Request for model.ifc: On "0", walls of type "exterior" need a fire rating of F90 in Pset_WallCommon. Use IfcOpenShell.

First a look at what the model holds.

```python
import ifcopenshell
import ifcopenshell.util.element

model = ifcopenshell.open("model.ifc")
print(model.schema)
storey = next(s for s in model.by_type("IfcBuildingStorey") if s.Name == "0")
walls = [e for e in ifcopenshell.util.element.get_decomposition(storey) if e.is_a("IfcWall")]
seen = {}
for e in walls:
    element_type = ifcopenshell.util.element.get_type(e)
    key = (element_type.Name if element_type != e and element_type else None, ifcopenshell.util.element.get_pset(e, "Pset_WallCommon", "FireRating"))
    seen[key] = seen.get(key, 0) + 1
for (name, value), count in sorted(seen.items(), key=str):
    print(count, "x", name, "|", value)
```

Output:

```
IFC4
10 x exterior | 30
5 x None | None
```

```python
import ifcopenshell
import ifcopenshell.api.pset
import ifcopenshell.util.element

model = ifcopenshell.open("model.ifc")

storey = next(s for s in model.by_type("IfcBuildingStorey") if s.Name == "0")
walls = [e for e in ifcopenshell.util.element.get_decomposition(storey) if e.is_a("IfcWall")]

count = 0
for e in walls:
    element_type = ifcopenshell.util.element.get_type(e)
    if element_type in (None, e) or element_type.Name != "exterior":
        continue
    # add_pset returns the element's existing set when there is one.
    pset = ifcopenshell.api.pset.add_pset(model, product=e, name="Pset_WallCommon")
    ifcopenshell.api.pset.edit_pset(model, pset=pset, properties={"FireRating": "F90"})
    count += 1

print(count, "walls updated")

model.write("model_v2.ifc")
```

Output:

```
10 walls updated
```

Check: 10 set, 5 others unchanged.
